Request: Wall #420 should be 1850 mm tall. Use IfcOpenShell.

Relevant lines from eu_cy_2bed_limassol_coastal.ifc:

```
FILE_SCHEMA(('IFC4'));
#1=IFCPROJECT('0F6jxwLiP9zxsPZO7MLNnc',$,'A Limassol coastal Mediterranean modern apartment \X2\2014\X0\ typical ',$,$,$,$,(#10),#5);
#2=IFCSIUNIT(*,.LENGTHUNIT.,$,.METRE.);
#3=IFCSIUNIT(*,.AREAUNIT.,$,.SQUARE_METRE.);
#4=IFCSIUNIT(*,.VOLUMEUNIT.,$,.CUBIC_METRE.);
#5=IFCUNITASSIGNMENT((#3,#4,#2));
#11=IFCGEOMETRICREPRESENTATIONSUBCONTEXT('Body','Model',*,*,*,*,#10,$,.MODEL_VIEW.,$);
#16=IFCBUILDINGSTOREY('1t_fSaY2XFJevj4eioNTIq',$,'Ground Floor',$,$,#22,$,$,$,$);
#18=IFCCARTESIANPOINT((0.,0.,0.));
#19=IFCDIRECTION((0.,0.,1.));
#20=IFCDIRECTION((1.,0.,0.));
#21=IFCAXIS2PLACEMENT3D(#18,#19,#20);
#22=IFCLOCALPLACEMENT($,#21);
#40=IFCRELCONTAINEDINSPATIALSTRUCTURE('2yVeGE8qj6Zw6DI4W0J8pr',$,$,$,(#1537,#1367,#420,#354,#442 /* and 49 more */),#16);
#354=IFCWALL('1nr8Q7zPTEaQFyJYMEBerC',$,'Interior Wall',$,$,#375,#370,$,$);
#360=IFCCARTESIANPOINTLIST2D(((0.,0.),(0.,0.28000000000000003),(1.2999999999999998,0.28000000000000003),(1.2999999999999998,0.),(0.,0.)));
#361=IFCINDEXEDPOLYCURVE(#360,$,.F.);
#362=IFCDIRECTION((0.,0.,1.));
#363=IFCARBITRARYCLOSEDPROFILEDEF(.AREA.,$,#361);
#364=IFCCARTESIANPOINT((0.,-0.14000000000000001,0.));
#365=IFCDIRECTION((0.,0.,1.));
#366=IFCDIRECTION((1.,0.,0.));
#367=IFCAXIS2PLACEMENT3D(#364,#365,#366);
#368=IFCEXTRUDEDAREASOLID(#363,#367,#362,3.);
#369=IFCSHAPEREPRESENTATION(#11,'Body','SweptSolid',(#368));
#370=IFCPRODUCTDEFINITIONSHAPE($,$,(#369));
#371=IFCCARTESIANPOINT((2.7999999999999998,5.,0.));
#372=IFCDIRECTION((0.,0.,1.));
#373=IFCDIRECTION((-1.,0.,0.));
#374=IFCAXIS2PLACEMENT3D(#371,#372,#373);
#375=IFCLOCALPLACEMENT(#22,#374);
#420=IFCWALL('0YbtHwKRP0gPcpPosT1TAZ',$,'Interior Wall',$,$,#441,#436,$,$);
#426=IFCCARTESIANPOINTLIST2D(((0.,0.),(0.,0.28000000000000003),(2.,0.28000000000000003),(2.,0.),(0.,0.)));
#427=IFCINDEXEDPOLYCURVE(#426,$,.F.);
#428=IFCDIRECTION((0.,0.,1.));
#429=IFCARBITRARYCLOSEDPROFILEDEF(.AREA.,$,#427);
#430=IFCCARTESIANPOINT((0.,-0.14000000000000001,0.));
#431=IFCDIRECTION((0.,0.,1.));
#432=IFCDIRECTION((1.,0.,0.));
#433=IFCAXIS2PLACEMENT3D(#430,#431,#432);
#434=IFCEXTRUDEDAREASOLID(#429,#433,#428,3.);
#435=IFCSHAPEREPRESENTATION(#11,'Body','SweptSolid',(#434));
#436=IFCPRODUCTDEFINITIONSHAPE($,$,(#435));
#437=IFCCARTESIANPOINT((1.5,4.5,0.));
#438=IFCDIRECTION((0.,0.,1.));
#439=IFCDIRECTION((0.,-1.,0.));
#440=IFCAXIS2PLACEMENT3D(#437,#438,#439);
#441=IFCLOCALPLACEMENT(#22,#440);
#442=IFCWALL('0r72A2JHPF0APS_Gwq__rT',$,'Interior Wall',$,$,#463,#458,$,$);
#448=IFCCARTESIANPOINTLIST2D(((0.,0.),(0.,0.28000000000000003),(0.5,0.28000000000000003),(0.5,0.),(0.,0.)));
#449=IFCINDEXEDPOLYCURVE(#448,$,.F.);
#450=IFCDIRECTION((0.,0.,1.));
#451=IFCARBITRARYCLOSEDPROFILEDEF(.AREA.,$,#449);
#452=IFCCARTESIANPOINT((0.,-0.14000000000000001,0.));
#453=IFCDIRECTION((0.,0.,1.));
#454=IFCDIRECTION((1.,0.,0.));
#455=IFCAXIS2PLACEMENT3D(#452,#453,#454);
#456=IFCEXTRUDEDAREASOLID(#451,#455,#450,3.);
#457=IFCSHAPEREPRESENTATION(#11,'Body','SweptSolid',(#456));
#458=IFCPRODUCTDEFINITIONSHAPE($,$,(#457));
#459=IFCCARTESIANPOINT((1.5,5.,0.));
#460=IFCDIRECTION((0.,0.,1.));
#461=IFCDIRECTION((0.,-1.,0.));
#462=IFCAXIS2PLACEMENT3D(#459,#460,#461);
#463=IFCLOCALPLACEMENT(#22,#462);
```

```python
import ifcopenshell
import ifcopenshell.geom
import ifcopenshell.util.representation
import ifcopenshell.util.shape
import ifcopenshell.util.unit

model = ifcopenshell.open("eu_cy_2bed_limassol_coastal.ifc")
unit_scale = ifcopenshell.util.unit.calculate_unit_scale(model)
settings = ifcopenshell.geom.settings()


def volume(element):
    """Net volume in cubic metres, openings subtracted."""
    shape = ifcopenshell.geom.create_shape(settings, element)
    return ifcopenshell.util.shape.get_volume(shape.geometry)


wall = model.by_id(420)
before = volume(wall)

body = ifcopenshell.util.representation.get_representation(wall, "Model", "Body")
solid = body.Items[0]
old_height = solid.Depth
solid.Depth = 1.85 / unit_scale
after = volume(wall)

print(f"height {old_height:g} -> {solid.Depth:g}, volume {before:.3f} -> {after:.3f} m3")

model.write("eu_cy_2bed_limassol_coastal_v2.ifc")
```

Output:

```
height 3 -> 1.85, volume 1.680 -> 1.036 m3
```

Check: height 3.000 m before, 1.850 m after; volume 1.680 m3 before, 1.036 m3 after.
